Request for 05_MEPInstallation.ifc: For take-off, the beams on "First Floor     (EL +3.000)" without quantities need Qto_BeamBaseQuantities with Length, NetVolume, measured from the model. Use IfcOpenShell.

First a look at what the model holds.

```python
import ifcopenshell
import ifcopenshell.util.element
import ifcopenshell.util.unit

model = ifcopenshell.open("05_MEPInstallation.ifc")
print(model.schema)
for unit_type in ("LENGTHUNIT", "AREAUNIT", "VOLUMEUNIT"):
    print(unit_type, ifcopenshell.util.unit.calculate_unit_scale(model, unit_type))
storey = next(s for s in model.by_type("IfcBuildingStorey") if s.Name == "First Floor     (EL +3.000)")
beams = [e for e in ifcopenshell.util.element.get_decomposition(storey) if e.is_a("IfcBeam")]
for e in sorted(beams, key=lambda e: e.id()):
    print(e.id(), e.is_a(), e.Name, list(ifcopenshell.util.element.get_psets(e, qtos_only=True)), sep=" | ")
```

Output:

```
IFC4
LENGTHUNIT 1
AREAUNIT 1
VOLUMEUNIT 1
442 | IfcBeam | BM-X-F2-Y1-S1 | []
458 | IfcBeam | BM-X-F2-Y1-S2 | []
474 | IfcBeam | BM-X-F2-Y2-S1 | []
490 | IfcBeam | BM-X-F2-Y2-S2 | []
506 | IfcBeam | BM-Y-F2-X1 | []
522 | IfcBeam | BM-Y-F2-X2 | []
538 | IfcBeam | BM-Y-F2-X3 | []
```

```python
import ifcopenshell
import ifcopenshell.api.pset
import ifcopenshell.geom
import ifcopenshell.util.element
import ifcopenshell.util.shape
import ifcopenshell.util.unit

model = ifcopenshell.open("05_MEPInstallation.ifc")
unit_scale = ifcopenshell.util.unit.calculate_unit_scale(model)
volume_scale = ifcopenshell.util.unit.calculate_unit_scale(model, "VOLUMEUNIT")
settings = ifcopenshell.geom.settings()

storey = next(s for s in model.by_type("IfcBuildingStorey") if s.Name == "First Floor     (EL +3.000)")
beams = [e for e in ifcopenshell.util.element.get_decomposition(storey) if e.is_a("IfcBeam")]

for e in sorted(beams, key=lambda e: e.id()):
    if ifcopenshell.util.element.get_psets(e, qtos_only=True, should_inherit=False):
        continue
    # Geometry comes back in metres, in the element's own axes.
    shape = ifcopenshell.geom.create_shape(settings, e)
    values = {
        "Length": ifcopenshell.util.shape.get_max_xyz(shape.geometry) / unit_scale,
        "NetVolume": ifcopenshell.util.shape.get_volume(shape.geometry) / volume_scale,
    }
    qto = ifcopenshell.api.pset.add_qto(model, product=e, name="Qto_BeamBaseQuantities")
    ifcopenshell.api.pset.edit_qto(model, qto=qto, properties=values)
    print(e.id(), {k: round(v, 3) for k, v in values.items()})

model.write("05_MEPInstallation_v2.ifc")
```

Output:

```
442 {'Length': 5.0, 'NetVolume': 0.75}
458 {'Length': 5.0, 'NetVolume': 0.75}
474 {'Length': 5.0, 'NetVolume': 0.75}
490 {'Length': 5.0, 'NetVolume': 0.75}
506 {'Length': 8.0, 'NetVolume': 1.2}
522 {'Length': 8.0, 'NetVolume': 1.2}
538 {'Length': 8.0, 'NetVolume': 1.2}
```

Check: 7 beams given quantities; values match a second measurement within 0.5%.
